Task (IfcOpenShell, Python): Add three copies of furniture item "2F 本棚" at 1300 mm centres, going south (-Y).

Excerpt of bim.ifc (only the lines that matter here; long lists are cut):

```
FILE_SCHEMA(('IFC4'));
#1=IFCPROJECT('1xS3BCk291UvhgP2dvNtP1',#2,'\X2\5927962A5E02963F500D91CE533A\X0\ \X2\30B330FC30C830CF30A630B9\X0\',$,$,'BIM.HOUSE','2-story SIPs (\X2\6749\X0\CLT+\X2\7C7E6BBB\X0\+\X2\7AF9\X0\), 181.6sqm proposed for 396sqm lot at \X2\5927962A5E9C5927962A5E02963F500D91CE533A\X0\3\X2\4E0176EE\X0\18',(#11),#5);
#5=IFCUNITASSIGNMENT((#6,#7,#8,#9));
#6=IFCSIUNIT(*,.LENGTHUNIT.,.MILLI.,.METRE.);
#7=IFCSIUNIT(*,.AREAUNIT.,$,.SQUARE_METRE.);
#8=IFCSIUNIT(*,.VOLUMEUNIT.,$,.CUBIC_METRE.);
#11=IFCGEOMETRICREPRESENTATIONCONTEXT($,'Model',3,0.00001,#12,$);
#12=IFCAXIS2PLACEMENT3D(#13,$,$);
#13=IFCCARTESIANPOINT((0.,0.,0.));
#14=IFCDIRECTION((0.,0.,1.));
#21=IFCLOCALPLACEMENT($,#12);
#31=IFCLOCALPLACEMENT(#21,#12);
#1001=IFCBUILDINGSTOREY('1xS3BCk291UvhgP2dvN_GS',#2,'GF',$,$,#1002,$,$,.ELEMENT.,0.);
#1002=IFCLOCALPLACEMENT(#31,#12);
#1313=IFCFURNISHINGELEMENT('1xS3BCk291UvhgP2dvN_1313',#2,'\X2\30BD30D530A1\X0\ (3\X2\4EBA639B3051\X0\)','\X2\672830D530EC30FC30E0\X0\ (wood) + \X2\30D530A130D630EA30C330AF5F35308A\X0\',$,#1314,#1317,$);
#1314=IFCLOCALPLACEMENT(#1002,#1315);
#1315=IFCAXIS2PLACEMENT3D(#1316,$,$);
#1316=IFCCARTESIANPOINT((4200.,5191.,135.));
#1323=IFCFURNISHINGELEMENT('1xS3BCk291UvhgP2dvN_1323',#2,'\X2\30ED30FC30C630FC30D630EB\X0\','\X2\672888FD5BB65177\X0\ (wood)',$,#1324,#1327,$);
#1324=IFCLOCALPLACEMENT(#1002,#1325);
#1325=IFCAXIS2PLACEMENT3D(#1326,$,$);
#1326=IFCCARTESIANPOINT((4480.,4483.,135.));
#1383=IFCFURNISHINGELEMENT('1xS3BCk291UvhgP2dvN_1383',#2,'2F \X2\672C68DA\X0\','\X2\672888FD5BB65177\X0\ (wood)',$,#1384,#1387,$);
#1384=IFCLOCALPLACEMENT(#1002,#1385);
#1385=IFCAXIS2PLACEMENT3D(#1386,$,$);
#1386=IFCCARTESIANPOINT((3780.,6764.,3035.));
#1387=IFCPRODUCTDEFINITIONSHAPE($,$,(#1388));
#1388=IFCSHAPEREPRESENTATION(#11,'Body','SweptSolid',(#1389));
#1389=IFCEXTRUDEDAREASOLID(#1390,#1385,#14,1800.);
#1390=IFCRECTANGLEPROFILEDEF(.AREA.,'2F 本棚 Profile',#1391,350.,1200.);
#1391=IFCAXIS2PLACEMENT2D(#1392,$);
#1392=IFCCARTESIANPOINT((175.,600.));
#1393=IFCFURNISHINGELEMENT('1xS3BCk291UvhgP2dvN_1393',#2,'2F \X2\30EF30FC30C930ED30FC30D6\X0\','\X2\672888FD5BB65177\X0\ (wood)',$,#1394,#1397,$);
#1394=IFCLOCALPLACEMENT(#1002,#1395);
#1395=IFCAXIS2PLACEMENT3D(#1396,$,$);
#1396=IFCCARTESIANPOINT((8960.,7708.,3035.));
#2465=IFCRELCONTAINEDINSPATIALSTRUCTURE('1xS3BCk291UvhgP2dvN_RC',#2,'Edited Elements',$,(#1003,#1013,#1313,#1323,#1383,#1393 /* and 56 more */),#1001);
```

```python
import numpy as np
import ifcopenshell
import ifcopenshell.api.geometry
import ifcopenshell.api.root
import ifcopenshell.util.element
import ifcopenshell.util.placement
import ifcopenshell.util.unit

model = ifcopenshell.open("bim.ifc")
unit_scale = ifcopenshell.util.unit.calculate_unit_scale(model)


def reuse_history(source, copy):
    """copy_class also copies each property set's owner history, people and application; keep the originals."""
    for rel in copy.IsDefinedBy:
        if rel.is_a("IfcRelDefinesByProperties") and (history := rel.RelatingPropertyDefinition.OwnerHistory):
            rel.RelatingPropertyDefinition.OwnerHistory = source.OwnerHistory
            ifcopenshell.util.element.remove_deep2(model, history)


source = model.by_guid("1xS3BCk291UvhgP2dvN_1383")
base = ifcopenshell.util.placement.get_local_placement(source.ObjectPlacement)
step = np.array([0.0, -1.0, 0.0]) * 1.3 / unit_scale

for i in range(1, 4):
    copy = ifcopenshell.api.root.copy_class(model, product=source)
    copy.Representation = ifcopenshell.util.element.copy_deep(
        model, source.Representation, exclude=["IfcGeometricRepresentationContext", "IfcRepresentationMap"]
    )
    reuse_history(source, copy)
    matrix = base.copy()
    matrix[:3, 3] += i * step
    print("added at", matrix[:3, 3].round(3) + 0.0)
    ifcopenshell.api.geometry.edit_object_placement(model, product=copy, matrix=matrix, is_si=False)

model.write("bim-out.ifc")
```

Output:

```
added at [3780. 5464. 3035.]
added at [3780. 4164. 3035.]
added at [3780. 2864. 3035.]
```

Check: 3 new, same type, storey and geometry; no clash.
